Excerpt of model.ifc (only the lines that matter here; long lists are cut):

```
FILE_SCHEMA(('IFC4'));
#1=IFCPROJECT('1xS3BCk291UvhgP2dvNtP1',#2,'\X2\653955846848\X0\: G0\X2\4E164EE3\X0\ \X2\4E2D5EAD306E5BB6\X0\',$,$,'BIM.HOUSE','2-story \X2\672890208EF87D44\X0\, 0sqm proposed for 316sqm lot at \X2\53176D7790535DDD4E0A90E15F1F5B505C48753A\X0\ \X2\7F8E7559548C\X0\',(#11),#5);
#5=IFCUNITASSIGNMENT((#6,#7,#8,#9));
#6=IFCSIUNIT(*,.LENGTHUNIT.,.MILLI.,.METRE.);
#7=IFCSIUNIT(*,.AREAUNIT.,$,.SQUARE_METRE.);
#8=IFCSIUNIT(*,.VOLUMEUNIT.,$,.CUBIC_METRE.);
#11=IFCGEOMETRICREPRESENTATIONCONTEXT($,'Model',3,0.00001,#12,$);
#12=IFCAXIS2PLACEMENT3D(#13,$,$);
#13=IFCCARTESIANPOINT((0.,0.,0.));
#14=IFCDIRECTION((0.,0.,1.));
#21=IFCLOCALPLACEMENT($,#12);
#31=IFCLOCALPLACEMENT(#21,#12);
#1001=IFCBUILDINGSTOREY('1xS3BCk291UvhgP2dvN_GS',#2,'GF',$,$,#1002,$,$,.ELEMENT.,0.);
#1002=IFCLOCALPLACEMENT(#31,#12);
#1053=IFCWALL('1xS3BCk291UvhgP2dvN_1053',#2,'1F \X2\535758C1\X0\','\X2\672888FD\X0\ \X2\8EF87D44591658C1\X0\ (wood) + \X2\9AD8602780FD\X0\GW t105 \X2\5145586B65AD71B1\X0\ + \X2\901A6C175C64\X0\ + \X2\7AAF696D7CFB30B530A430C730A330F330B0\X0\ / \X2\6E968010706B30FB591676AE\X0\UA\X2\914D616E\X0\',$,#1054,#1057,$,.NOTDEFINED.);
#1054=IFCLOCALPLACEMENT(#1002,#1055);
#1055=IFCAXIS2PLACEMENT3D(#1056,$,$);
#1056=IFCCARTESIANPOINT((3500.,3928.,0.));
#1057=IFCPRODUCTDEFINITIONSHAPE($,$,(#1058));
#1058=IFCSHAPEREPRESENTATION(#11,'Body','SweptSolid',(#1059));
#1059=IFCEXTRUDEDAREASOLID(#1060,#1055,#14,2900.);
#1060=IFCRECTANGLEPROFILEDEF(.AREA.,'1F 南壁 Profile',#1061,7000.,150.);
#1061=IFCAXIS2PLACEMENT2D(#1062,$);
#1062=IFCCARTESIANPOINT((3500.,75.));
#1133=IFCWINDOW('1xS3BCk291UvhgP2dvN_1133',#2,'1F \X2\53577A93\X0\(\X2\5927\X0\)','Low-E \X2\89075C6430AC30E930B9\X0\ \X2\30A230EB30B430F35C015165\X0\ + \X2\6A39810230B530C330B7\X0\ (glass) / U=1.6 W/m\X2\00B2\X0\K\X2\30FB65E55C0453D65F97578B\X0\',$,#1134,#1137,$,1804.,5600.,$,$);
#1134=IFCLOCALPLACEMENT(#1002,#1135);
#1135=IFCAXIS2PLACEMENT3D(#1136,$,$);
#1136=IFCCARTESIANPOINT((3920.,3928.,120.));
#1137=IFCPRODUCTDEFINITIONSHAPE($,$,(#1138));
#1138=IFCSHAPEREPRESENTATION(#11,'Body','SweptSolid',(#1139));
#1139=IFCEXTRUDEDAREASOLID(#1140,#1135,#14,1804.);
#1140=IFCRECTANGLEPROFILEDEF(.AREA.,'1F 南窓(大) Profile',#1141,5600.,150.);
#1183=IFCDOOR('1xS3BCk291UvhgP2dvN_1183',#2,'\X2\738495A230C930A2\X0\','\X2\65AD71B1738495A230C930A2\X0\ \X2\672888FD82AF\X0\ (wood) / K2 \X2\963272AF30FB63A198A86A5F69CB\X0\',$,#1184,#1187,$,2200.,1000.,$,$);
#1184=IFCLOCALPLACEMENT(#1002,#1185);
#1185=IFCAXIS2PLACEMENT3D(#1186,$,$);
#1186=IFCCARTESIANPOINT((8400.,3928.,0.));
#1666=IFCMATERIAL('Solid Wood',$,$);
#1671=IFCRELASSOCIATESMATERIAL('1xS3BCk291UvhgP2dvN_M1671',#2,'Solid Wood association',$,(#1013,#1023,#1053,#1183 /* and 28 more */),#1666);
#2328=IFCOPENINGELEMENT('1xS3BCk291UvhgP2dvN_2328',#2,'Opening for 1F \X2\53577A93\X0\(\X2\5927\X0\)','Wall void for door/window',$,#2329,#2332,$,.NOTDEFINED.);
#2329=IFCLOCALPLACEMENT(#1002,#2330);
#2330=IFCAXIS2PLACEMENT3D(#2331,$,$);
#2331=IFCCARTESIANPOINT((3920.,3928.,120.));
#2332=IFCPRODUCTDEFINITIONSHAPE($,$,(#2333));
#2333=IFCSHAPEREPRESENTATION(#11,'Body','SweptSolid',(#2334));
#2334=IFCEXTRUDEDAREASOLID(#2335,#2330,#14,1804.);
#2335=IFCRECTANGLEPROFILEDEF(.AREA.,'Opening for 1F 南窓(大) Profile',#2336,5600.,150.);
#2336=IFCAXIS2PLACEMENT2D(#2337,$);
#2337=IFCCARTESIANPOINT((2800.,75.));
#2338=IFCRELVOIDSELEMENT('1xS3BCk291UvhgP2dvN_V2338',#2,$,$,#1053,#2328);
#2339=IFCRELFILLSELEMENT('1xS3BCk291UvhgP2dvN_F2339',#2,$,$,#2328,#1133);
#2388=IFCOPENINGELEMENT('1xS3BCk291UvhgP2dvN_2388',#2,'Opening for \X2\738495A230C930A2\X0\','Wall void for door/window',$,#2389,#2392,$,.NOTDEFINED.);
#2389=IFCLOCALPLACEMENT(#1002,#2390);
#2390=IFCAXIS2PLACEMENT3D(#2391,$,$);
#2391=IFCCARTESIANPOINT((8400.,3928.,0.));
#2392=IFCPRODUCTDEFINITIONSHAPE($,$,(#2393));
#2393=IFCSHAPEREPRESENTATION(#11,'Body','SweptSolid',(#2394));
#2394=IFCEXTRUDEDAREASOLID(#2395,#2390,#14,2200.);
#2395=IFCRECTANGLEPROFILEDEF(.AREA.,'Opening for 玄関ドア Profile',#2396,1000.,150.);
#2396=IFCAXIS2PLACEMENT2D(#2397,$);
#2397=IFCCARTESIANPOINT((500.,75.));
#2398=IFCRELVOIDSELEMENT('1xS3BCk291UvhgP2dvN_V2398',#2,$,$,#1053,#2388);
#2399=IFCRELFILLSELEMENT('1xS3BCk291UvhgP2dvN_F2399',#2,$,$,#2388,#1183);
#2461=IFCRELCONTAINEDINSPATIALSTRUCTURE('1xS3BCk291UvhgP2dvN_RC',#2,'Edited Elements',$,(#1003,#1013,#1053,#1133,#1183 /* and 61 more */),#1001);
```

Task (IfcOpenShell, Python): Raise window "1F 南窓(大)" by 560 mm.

```python
import numpy as np
import ifcopenshell
import ifcopenshell.api.geometry
import ifcopenshell.util.placement
import ifcopenshell.util.unit

model = ifcopenshell.open("model.ifc")
unit_scale = ifcopenshell.util.unit.calculate_unit_scale(model)

window = model.by_guid("1xS3BCk291UvhgP2dvN_1133")
opening = window.FillsVoids[0].RelatingOpeningElement
dz = 0.56 / unit_scale

shift = np.array([0.0, 0.0, dz])
# The window is not placed relative to its opening, so move both.
for product in (opening, window):
    matrix = ifcopenshell.util.placement.get_local_placement(product.ObjectPlacement)
    matrix[:3, 3] += shift
    ifcopenshell.api.geometry.edit_object_placement(model, product=product, matrix=matrix, is_si=False)

print(f"moved by {dz * unit_scale:+.3f} m")

model.write("model-out.ifc")
```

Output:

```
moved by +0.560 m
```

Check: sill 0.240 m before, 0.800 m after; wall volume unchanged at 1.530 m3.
